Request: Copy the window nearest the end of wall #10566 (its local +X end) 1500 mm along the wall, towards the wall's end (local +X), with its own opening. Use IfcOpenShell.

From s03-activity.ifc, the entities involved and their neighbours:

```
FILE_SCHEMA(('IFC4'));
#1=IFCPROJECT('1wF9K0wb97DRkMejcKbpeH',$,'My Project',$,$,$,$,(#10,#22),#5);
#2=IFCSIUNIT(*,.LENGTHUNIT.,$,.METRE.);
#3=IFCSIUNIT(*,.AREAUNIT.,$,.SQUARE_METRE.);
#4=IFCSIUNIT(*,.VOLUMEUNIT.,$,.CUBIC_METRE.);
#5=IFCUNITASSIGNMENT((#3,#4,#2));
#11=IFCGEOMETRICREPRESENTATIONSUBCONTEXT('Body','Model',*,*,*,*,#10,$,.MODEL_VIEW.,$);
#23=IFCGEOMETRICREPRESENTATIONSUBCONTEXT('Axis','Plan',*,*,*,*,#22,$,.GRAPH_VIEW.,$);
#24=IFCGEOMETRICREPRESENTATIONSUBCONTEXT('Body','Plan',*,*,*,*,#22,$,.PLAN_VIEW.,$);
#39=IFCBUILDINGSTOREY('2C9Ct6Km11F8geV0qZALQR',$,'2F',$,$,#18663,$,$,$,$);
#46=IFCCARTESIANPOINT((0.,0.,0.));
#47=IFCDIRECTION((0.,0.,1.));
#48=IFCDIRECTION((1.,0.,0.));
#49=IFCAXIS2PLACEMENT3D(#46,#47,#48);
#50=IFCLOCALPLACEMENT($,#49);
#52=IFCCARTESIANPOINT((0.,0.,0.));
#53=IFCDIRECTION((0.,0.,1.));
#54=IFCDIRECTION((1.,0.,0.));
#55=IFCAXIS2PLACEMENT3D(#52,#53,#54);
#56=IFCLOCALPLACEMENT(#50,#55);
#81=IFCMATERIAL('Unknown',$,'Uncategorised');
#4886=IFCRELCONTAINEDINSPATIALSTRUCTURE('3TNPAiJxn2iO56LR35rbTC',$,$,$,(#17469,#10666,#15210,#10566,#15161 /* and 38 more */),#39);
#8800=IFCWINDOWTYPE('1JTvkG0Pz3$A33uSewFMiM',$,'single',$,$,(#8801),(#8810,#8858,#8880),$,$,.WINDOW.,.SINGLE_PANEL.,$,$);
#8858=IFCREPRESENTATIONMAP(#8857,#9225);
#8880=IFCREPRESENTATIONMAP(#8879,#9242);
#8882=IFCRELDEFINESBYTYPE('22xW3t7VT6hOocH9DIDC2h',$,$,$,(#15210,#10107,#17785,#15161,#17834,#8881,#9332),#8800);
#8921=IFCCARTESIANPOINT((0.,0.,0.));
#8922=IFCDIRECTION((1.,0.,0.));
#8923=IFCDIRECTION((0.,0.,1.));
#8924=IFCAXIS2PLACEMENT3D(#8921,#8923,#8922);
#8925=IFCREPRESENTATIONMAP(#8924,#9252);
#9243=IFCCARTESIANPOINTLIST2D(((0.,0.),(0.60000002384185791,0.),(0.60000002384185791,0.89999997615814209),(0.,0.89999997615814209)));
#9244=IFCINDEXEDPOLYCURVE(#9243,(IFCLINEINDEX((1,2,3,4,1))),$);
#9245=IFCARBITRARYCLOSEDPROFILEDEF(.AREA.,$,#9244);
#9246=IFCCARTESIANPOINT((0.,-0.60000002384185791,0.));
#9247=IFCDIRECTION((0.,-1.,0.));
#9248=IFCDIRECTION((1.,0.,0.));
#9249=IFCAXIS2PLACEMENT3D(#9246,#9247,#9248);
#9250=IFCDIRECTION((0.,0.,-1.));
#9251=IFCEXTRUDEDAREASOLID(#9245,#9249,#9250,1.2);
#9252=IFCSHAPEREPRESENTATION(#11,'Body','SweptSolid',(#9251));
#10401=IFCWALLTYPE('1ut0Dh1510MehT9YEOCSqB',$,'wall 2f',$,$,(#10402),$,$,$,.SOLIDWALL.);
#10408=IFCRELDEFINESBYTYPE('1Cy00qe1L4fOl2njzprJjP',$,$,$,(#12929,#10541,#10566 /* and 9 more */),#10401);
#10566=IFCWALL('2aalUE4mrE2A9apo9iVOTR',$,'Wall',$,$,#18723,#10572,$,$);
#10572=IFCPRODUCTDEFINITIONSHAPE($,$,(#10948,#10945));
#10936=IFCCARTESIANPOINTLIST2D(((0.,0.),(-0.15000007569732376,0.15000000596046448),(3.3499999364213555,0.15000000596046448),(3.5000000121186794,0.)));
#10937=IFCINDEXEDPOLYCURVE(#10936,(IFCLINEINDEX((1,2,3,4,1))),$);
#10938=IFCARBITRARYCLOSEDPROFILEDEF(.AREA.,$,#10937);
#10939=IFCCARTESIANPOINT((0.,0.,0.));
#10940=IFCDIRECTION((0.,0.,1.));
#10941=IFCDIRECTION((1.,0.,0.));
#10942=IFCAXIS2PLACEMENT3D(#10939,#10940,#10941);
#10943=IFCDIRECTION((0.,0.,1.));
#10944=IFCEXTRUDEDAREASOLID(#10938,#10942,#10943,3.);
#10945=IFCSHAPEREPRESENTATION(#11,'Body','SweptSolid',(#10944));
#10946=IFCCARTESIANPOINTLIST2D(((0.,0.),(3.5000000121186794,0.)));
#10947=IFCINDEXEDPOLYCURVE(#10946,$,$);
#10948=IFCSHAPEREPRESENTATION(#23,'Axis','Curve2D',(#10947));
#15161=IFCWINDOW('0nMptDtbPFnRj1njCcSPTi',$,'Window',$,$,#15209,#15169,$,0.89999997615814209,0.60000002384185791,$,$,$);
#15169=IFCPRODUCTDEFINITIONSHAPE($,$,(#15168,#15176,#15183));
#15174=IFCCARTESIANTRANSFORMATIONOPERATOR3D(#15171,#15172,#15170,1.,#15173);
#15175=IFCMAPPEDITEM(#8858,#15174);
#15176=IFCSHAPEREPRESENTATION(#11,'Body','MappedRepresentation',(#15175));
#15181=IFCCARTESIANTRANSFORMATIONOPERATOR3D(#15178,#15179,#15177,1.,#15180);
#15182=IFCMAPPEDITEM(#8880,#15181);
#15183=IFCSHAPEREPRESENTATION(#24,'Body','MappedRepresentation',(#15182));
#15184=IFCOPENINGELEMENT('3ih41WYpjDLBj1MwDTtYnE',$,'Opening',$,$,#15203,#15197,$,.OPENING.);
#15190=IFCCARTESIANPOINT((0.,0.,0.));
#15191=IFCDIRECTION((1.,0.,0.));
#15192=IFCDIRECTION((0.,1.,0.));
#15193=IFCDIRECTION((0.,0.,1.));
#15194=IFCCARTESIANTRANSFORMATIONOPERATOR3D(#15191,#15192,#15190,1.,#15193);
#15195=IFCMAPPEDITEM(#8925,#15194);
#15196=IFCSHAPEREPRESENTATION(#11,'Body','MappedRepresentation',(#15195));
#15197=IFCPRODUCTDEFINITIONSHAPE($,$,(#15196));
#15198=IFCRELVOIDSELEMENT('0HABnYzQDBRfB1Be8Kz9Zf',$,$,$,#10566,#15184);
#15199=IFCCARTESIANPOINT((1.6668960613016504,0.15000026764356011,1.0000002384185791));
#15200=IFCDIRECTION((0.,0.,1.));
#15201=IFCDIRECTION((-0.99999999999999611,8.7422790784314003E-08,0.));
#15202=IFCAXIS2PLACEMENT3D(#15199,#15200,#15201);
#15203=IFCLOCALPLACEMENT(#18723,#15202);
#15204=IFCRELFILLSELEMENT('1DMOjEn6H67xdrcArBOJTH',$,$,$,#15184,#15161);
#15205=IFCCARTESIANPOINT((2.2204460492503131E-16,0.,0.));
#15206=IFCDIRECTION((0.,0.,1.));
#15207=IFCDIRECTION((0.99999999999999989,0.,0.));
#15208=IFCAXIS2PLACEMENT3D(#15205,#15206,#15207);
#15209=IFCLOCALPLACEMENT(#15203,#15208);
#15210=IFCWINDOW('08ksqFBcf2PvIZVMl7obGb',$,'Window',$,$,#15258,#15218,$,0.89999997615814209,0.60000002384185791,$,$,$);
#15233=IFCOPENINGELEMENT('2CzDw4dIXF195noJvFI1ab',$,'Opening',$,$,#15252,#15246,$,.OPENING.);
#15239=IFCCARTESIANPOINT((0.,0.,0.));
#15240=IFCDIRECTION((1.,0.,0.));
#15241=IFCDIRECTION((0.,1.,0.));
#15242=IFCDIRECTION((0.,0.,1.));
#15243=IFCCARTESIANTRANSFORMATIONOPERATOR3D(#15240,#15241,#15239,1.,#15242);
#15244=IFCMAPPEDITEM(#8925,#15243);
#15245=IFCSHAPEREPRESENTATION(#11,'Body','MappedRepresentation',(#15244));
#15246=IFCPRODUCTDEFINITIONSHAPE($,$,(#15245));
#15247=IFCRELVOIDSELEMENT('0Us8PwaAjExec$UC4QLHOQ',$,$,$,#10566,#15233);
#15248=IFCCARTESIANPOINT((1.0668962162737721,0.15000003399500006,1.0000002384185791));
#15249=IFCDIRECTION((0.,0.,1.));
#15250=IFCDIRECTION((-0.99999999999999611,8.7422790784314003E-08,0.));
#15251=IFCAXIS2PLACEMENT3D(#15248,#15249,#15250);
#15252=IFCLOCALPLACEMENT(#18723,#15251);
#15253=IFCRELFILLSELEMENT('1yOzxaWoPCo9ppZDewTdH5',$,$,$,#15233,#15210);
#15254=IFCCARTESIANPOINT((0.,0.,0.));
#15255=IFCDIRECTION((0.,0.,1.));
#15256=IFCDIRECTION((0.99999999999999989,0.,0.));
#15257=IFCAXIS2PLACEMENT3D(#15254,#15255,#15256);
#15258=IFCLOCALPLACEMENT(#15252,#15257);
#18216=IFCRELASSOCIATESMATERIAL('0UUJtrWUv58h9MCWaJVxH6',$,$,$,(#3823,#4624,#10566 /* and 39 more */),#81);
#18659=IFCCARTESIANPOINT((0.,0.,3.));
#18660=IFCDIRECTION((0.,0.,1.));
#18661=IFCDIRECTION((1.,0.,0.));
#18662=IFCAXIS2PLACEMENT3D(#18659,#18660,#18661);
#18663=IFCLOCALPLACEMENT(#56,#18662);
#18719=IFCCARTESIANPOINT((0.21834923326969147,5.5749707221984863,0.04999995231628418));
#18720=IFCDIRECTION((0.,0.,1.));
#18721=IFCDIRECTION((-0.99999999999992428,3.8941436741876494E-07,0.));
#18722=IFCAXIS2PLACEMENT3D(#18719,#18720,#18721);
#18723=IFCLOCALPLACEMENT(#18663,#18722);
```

```python
import ifcopenshell
import ifcopenshell.api.feature
import ifcopenshell.api.geometry
import ifcopenshell.api.root
import ifcopenshell.geom
import ifcopenshell.util.element
import ifcopenshell.util.placement
import ifcopenshell.util.shape
import ifcopenshell.util.unit

model = ifcopenshell.open("s03-activity.ifc")
unit_scale = ifcopenshell.util.unit.calculate_unit_scale(model)
settings = ifcopenshell.geom.settings()


def volume(element):
    """Net volume in cubic metres, openings subtracted."""
    shape = ifcopenshell.geom.create_shape(settings, element)
    return ifcopenshell.util.shape.get_volume(shape.geometry)


window = model.by_guid("0nMptDtbPFnRj1njCcSPTi")
opening = window.FillsVoids[0].RelatingOpeningElement
wall = opening.VoidsElements[0].RelatingBuildingElement
before = volume(wall)
shift = ifcopenshell.util.placement.get_local_placement(wall.ObjectPlacement)[:3, 0] * 1.5 / unit_scale

# copy_class copies the void relationship, type, container and properties, but no geometry.
new_opening = ifcopenshell.api.root.copy_class(model, product=opening)
new_opening.Representation = ifcopenshell.util.element.copy_deep(
    model, opening.Representation, exclude=["IfcGeometricRepresentationContext", "IfcRepresentationMap"]
)
new_window = ifcopenshell.api.root.copy_class(model, product=window)
new_window.Representation = ifcopenshell.util.element.copy_deep(
    model, window.Representation, exclude=["IfcGeometricRepresentationContext", "IfcRepresentationMap"]
)
ifcopenshell.api.feature.add_filling(model, opening=new_opening, element=new_window)

for old, new in ((opening, new_opening), (window, new_window)):
    matrix = ifcopenshell.util.placement.get_local_placement(old.ObjectPlacement)
    matrix[:3, 3] += shift
    ifcopenshell.api.geometry.edit_object_placement(model, product=new, matrix=matrix, is_si=False)

after = volume(wall)

print(f"wall volume {before:.3f} -> {after:.3f} m3")

model.write("s03-activity_edited.ifc")
```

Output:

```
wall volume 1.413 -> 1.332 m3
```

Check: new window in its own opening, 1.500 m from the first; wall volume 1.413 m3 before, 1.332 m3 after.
